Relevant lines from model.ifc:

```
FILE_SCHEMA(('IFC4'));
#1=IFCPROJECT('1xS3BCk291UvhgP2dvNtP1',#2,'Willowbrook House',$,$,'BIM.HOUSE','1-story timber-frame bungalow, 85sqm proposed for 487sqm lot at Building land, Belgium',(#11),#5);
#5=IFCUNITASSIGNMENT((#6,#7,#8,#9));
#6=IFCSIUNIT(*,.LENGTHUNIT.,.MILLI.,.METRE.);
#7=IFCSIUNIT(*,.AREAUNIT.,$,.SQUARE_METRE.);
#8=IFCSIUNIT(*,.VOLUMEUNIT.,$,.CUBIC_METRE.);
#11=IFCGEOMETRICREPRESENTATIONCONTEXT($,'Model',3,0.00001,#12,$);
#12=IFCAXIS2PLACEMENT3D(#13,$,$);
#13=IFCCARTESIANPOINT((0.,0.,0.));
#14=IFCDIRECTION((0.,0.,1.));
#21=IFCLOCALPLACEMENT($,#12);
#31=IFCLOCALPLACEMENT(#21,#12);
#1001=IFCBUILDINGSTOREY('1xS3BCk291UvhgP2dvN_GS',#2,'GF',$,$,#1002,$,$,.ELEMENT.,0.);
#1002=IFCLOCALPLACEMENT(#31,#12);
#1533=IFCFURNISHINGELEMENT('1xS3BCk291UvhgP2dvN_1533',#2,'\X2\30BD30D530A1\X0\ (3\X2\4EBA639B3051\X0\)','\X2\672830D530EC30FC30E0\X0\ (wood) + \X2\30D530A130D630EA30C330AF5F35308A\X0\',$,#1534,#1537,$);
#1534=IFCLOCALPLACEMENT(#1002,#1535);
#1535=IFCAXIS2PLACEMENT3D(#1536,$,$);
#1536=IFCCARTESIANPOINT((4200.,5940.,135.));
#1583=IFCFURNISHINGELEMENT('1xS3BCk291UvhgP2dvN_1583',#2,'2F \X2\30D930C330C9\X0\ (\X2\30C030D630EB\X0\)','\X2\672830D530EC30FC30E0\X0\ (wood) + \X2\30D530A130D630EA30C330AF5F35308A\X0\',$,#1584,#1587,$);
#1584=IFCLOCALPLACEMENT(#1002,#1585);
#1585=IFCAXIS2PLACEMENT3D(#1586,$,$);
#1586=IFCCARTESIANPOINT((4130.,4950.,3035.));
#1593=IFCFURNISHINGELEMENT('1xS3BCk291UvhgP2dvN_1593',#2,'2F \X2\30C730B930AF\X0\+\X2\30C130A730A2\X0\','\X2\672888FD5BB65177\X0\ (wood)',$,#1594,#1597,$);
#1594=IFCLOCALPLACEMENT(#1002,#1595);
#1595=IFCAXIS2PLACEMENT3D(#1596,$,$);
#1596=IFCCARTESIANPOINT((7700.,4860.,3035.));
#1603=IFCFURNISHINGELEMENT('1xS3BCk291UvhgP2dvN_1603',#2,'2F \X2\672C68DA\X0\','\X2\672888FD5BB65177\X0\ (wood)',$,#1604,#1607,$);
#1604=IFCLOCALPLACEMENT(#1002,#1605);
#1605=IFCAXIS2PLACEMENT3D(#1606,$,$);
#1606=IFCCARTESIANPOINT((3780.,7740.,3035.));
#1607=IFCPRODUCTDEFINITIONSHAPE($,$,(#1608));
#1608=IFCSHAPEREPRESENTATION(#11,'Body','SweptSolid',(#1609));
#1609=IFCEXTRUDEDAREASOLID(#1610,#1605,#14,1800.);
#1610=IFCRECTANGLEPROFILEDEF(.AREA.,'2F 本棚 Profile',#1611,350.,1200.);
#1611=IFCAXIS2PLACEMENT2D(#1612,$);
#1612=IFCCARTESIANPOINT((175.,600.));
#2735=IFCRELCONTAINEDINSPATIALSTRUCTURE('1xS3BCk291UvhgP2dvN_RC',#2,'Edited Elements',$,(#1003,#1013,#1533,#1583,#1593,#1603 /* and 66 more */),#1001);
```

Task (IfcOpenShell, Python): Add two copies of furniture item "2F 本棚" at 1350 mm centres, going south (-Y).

```python
import numpy as np
import ifcopenshell
import ifcopenshell.api.geometry
import ifcopenshell.api.root
import ifcopenshell.util.element
import ifcopenshell.util.placement
import ifcopenshell.util.unit

model = ifcopenshell.open("model.ifc")
unit_scale = ifcopenshell.util.unit.calculate_unit_scale(model)


def reuse_history(source, copy):
    """copy_class also copies each property set's owner history, people and application; keep the originals."""
    for rel in copy.IsDefinedBy:
        if rel.is_a("IfcRelDefinesByProperties") and (history := rel.RelatingPropertyDefinition.OwnerHistory):
            rel.RelatingPropertyDefinition.OwnerHistory = source.OwnerHistory
            ifcopenshell.util.element.remove_deep2(model, history)


source = model.by_guid("1xS3BCk291UvhgP2dvN_1603")
base = ifcopenshell.util.placement.get_local_placement(source.ObjectPlacement)
step = np.array([0.0, -1.0, 0.0]) * 1.35 / unit_scale

for i in range(1, 3):
    copy = ifcopenshell.api.root.copy_class(model, product=source)
    copy.Representation = ifcopenshell.util.element.copy_deep(
        model, source.Representation, exclude=["IfcGeometricRepresentationContext", "IfcRepresentationMap"]
    )
    reuse_history(source, copy)
    matrix = base.copy()
    matrix[:3, 3] += i * step
    print("added at", matrix[:3, 3].round(3) + 0.0)
    ifcopenshell.api.geometry.edit_object_placement(model, product=copy, matrix=matrix, is_si=False)

model.write("model_v2.ifc")
```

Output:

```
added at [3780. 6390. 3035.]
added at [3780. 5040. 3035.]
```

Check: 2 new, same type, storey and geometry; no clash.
